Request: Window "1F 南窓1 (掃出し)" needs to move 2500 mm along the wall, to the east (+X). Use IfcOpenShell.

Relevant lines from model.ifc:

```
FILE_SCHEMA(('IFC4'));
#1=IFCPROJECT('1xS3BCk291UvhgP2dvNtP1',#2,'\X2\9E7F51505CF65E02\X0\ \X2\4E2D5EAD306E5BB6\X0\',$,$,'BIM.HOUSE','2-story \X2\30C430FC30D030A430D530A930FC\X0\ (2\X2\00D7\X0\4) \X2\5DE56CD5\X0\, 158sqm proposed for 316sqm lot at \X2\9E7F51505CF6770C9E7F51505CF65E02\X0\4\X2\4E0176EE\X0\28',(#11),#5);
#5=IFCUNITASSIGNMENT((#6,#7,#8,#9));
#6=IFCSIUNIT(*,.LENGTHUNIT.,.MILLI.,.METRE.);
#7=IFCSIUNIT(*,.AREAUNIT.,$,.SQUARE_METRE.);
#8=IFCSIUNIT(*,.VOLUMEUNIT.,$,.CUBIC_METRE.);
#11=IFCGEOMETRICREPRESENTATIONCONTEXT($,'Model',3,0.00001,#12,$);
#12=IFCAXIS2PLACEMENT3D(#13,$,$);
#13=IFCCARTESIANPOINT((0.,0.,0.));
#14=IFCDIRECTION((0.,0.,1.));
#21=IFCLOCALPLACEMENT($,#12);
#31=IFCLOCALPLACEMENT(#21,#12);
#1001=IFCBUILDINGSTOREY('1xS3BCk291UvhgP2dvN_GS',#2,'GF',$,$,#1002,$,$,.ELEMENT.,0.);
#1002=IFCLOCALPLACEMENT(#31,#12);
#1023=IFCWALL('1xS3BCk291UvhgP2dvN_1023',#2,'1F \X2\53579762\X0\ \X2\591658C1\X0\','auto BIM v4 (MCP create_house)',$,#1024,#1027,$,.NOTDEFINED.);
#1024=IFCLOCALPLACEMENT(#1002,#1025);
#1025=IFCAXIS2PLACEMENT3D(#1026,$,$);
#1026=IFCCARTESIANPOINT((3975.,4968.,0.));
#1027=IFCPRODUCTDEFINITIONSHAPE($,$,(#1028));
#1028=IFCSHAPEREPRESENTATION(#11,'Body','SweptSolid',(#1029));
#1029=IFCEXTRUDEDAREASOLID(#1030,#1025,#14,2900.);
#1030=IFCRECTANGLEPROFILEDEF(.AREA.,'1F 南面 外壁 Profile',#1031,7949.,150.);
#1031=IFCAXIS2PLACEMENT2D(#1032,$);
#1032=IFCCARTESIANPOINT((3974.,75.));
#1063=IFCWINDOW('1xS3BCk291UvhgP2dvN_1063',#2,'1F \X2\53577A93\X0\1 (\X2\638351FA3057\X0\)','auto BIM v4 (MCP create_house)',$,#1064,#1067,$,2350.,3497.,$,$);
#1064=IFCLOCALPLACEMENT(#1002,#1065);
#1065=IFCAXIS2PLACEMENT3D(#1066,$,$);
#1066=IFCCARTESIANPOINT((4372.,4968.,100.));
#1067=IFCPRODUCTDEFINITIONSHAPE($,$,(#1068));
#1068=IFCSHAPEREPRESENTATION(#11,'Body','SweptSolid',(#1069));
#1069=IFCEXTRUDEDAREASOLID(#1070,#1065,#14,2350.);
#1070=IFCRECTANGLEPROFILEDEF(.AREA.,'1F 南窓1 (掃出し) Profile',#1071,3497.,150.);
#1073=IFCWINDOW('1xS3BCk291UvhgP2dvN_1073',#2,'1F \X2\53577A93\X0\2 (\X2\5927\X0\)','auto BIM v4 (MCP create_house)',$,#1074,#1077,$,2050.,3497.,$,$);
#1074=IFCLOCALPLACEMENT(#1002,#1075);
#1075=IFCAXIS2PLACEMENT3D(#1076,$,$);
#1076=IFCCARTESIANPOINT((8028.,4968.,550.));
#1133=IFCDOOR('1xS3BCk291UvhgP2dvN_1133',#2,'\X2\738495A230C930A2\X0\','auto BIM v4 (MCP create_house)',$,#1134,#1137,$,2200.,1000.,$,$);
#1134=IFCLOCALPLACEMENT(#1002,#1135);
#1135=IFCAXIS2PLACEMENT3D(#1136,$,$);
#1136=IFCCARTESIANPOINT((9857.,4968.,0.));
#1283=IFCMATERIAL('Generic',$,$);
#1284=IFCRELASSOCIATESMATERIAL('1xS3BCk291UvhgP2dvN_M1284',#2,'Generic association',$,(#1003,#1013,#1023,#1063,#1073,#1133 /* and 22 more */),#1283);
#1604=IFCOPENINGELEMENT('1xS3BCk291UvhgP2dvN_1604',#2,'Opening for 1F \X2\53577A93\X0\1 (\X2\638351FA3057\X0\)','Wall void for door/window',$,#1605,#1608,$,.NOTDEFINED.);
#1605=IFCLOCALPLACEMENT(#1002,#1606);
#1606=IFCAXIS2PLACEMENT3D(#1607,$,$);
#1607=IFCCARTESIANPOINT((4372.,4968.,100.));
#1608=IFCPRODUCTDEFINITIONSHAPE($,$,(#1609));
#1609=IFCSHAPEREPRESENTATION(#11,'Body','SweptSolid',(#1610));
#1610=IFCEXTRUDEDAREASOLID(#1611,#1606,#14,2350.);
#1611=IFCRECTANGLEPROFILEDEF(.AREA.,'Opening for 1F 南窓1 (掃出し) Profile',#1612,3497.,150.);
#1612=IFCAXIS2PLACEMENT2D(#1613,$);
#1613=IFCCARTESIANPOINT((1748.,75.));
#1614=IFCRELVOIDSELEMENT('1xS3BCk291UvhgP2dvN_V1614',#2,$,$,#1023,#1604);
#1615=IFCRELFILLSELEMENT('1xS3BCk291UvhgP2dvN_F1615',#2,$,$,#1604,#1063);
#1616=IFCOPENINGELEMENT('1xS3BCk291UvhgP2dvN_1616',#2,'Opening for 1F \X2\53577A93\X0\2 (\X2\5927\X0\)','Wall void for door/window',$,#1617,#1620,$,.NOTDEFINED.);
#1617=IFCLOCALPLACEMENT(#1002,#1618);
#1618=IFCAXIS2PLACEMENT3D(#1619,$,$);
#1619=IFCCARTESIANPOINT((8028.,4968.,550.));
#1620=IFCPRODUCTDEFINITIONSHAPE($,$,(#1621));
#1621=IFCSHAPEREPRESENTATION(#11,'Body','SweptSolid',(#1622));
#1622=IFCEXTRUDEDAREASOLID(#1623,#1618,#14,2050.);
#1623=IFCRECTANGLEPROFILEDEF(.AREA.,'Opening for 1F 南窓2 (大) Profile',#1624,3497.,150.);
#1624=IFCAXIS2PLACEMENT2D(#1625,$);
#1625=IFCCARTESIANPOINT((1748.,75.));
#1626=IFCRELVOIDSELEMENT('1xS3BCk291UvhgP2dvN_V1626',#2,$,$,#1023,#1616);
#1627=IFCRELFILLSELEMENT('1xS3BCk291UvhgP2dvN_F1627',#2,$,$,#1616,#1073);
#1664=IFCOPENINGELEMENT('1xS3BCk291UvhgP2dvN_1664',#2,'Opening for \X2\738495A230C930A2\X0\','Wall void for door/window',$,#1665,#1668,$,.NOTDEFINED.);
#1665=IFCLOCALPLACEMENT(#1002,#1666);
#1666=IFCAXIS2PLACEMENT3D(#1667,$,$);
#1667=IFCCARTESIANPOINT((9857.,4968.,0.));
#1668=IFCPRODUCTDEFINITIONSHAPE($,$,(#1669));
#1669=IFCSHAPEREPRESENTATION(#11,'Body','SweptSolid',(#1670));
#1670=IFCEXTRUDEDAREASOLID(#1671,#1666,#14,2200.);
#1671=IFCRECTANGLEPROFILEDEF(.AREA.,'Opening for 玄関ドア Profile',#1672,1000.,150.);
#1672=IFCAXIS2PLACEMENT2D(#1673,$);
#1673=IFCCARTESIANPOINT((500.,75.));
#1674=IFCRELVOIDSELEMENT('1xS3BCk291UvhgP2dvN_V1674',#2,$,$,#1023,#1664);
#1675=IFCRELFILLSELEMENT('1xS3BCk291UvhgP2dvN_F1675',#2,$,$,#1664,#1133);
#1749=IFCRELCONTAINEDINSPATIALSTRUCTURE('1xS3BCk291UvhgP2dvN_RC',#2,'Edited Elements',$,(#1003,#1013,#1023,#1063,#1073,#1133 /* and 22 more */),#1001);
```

```python
import ifcopenshell
import ifcopenshell.api.geometry
import ifcopenshell.util.placement
import ifcopenshell.util.unit

model = ifcopenshell.open("model.ifc")
unit_scale = ifcopenshell.util.unit.calculate_unit_scale(model)

window = model.by_guid("1xS3BCk291UvhgP2dvN_1063")
opening = window.FillsVoids[0].RelatingOpeningElement
wall = opening.VoidsElements[0].RelatingBuildingElement

wall_matrix = ifcopenshell.util.placement.get_local_placement(wall.ObjectPlacement)
shift = wall_matrix[:3, 0] * 2.5 / unit_scale
before = ifcopenshell.util.placement.get_local_placement(window.ObjectPlacement)[:3, 3].copy()

# The window is not placed relative to its opening, so move both.
for product in (opening, window):
    matrix = ifcopenshell.util.placement.get_local_placement(product.ObjectPlacement)
    matrix[:3, 3] += shift
    ifcopenshell.api.geometry.edit_object_placement(model, product=product, matrix=matrix, is_si=False)

after = ifcopenshell.util.placement.get_local_placement(window.ObjectPlacement)[:3, 3]
print("window moved by", (after - before).round(3) + 0.0)

model.write("model_rev.ifc")
```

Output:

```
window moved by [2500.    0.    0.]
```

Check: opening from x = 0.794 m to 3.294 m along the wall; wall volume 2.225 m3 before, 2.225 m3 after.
